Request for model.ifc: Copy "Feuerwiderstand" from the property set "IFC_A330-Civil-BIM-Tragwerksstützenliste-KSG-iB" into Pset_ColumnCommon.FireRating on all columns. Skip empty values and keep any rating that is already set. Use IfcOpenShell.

First a look at what the model holds.

```python
import ifcopenshell
import ifcopenshell.util.element

model = ifcopenshell.open("model.ifc")
print(model.schema)
columns = model.by_type("IfcColumn")
print(len(columns), "columns")
for e in columns[:8]:
    source = ifcopenshell.util.element.get_pset(e, "IFC_A330-Civil-BIM-Tragwerksstützenliste-KSG-iB", "Feuerwiderstand")
    target = ifcopenshell.util.element.get_pset(e, "Pset_ColumnCommon", "FireRating")
    print(e.id(), repr(source), repr(target), sep=" | ")
```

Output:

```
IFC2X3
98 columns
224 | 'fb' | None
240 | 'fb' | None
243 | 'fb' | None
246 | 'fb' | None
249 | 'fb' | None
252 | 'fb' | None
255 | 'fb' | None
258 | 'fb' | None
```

```python
import ifcopenshell
import ifcopenshell.api.pset
import ifcopenshell.util.element

model = ifcopenshell.open("model.ifc")

count = 0
for e in model.by_type("IfcColumn"):
    value = ifcopenshell.util.element.get_pset(e, "IFC_A330-Civil-BIM-Tragwerksstützenliste-KSG-iB", "Feuerwiderstand")
    current = ifcopenshell.util.element.get_pset(e, "Pset_ColumnCommon", "FireRating")
    if not value or not value.strip() or current:
        continue
    found = ifcopenshell.util.element.get_pset(e, "Pset_ColumnCommon", should_inherit=False)
    if found:
        pset = model.by_id(found["id"])
        if len(ifcopenshell.util.element.get_elements_by_pset(pset)) > 1:
            pset = ifcopenshell.api.pset.unshare_pset(model, products=[e], pset=pset)[0]
    else:
        pset = ifcopenshell.api.pset.add_pset(model, product=e, name="Pset_ColumnCommon")
    ifcopenshell.api.pset.edit_pset(model, pset=pset, properties={"FireRating": value})
    count += 1

print(count, "columns updated")

model.write("model_edited.ifc")
```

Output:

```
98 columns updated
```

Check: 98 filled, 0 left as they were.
